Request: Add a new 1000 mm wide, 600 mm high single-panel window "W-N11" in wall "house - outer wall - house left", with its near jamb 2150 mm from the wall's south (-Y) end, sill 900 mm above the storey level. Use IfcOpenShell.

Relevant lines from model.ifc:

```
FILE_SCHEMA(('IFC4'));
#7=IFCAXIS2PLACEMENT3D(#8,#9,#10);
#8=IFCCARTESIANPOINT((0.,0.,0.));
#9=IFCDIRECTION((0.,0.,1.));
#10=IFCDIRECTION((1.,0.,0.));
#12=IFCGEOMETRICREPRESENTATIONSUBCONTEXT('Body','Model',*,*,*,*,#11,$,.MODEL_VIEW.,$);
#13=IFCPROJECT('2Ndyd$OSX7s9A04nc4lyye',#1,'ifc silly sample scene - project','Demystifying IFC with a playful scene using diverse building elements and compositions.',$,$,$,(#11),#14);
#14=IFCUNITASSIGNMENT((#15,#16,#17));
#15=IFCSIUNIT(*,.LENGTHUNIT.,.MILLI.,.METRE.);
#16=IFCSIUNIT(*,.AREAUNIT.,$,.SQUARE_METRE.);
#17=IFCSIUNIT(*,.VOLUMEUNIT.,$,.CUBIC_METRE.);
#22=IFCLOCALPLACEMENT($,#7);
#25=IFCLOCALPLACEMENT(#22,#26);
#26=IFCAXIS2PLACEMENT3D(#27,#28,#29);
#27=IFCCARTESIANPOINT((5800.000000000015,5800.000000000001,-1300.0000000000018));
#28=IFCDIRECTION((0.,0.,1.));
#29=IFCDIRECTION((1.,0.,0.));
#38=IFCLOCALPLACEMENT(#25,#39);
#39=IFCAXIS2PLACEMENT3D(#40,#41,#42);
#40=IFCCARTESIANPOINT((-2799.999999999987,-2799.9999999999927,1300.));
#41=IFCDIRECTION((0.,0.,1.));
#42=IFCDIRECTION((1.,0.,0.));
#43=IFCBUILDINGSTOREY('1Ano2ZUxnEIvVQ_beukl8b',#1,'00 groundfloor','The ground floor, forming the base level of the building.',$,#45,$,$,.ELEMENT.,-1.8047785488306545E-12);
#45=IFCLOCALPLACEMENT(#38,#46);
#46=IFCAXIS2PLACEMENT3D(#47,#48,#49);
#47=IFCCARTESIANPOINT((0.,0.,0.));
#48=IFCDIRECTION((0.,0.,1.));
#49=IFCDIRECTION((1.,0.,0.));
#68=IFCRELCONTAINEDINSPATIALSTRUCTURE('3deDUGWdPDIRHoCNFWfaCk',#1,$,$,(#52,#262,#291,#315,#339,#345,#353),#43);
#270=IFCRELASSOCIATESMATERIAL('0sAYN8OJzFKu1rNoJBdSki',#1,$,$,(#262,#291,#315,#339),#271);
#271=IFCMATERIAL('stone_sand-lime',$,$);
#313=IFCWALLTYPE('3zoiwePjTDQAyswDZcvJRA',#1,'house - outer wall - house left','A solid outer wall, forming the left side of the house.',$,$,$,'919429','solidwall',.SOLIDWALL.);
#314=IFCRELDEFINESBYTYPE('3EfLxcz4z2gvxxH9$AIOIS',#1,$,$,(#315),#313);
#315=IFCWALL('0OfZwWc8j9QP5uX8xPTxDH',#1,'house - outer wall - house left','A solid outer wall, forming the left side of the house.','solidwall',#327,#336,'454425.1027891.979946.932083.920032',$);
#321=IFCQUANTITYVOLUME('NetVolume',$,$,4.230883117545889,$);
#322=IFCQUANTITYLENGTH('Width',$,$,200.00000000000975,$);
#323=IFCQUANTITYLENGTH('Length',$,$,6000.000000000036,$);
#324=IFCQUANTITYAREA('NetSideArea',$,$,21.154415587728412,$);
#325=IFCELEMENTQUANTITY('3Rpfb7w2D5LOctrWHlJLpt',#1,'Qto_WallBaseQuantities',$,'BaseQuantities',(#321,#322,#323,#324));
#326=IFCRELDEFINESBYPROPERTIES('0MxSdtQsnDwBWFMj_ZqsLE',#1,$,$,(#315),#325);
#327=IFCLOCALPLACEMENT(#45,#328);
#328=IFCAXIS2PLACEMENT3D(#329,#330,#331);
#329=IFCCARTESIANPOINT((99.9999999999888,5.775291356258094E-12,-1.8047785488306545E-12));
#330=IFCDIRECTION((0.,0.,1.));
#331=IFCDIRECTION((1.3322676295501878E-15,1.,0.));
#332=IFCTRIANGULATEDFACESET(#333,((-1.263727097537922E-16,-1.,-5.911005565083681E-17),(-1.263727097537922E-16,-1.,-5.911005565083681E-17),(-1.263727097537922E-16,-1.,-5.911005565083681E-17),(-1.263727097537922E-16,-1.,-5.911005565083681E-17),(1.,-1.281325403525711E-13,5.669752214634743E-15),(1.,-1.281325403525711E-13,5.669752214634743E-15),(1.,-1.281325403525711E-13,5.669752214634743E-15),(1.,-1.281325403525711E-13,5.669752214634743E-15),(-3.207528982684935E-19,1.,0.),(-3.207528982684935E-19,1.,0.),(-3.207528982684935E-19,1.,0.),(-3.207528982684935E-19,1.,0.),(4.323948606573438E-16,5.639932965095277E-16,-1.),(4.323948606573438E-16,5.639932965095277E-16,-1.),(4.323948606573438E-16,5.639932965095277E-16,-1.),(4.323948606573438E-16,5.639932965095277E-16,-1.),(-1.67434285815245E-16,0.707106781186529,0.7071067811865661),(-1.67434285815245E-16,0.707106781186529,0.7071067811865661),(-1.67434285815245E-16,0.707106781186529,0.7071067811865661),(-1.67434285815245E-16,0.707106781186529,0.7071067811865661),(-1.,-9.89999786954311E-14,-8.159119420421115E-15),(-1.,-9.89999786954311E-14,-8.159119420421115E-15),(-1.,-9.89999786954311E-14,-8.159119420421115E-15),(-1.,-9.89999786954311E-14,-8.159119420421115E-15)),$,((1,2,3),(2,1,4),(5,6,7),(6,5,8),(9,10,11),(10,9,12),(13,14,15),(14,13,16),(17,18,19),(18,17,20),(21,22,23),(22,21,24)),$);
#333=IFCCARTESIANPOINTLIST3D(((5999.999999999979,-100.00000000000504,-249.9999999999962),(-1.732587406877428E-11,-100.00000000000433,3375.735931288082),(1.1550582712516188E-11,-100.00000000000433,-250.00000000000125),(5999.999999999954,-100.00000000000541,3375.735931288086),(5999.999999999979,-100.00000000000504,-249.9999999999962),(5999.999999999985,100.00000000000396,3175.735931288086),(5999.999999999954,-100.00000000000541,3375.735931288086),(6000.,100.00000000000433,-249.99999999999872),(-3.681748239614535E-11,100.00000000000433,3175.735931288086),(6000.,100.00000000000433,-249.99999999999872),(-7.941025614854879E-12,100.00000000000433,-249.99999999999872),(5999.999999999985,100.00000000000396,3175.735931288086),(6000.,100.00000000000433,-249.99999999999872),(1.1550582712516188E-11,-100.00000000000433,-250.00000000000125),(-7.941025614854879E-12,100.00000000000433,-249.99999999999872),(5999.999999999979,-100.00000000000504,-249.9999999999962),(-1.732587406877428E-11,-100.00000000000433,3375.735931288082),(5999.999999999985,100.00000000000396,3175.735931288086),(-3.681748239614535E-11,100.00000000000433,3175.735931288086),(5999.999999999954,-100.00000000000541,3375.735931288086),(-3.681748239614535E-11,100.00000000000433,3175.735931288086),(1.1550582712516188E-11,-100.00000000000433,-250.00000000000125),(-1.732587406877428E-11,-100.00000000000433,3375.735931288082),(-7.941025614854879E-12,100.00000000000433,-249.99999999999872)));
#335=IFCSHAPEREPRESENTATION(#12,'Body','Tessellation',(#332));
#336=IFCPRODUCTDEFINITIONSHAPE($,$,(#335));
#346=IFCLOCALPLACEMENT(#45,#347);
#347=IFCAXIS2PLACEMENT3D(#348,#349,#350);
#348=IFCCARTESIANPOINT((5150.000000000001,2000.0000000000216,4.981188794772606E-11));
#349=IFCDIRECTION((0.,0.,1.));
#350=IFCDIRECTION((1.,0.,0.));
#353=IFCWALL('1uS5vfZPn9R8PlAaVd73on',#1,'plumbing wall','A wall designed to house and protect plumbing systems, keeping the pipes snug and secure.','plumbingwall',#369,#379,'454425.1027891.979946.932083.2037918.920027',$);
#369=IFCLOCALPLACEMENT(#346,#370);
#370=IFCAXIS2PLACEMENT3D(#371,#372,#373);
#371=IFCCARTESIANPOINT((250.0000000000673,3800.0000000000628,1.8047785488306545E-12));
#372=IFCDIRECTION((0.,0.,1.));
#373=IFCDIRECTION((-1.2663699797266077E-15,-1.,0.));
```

```python
import numpy as np
import ifcopenshell
import ifcopenshell.api.feature
import ifcopenshell.api.geometry
import ifcopenshell.api.pset
import ifcopenshell.api.root
import ifcopenshell.api.spatial
import ifcopenshell.geom
import ifcopenshell.util.element
import ifcopenshell.util.placement
import ifcopenshell.util.representation
import ifcopenshell.util.shape
import ifcopenshell.util.unit

model = ifcopenshell.open("model.ifc")
unit_scale = ifcopenshell.util.unit.calculate_unit_scale(model)
area_scale = ifcopenshell.util.unit.calculate_unit_scale(model, "AREAUNIT")
volume_scale = ifcopenshell.util.unit.calculate_unit_scale(model, "VOLUMEUNIT")
settings = ifcopenshell.geom.settings()


def volume(element):
    """Net volume in cubic metres, openings subtracted."""
    shape = ifcopenshell.geom.create_shape(settings, element)
    return ifcopenshell.util.shape.get_volume(shape.geometry)


wall = model.by_guid("0OfZwWc8j9QP5uX8xPTxDH")
storey = ifcopenshell.util.element.get_container(wall, ifc_class="IfcBuildingStorey")
context = ifcopenshell.util.representation.get_context(model, "Model", "Body", "MODEL_VIEW")
before = volume(wall)

width, height, from_end, sill = 1, 0.6, 2.15, 0.9  # metres

# The wall runs along its own X axis, and the end named is its -X end.
wall_shape = ifcopenshell.geom.create_shape(settings, wall)
x, y, z = ifcopenshell.util.shape.get_vertices(wall_shape.geometry).T
start = x.min() + from_end
face, thickness = float(y.min()), float(y.max() - y.min())
wall_matrix = ifcopenshell.util.placement.get_local_placement(wall.ObjectPlacement)
level = ifcopenshell.util.placement.get_local_placement(storey.ObjectPlacement)[2, 3]


def in_wall(x, y):
    """Placement at x, y metres in the wall's axes, at sill height."""
    matrix = wall_matrix.copy()
    matrix[:, 3] = wall_matrix @ np.array([x / unit_scale, y / unit_scale, 0.0, 1.0])
    matrix[2, 3] = level + sill / unit_scale
    return matrix


# Opening: a box that overshoots both wall faces by 50 mm.
opening = ifcopenshell.api.root.create_entity(model, ifc_class="IfcOpeningElement", predefined_type="OPENING")
box = ifcopenshell.api.geometry.add_wall_representation(
    model, context=context, length=width, height=height, thickness=thickness + 0.1
)
ifcopenshell.api.geometry.assign_representation(model, product=opening, representation=box)
ifcopenshell.api.geometry.edit_object_placement(model, product=opening, matrix=in_wall(start, face - 0.05), is_si=False)
ifcopenshell.api.feature.add_feature(model, feature=opening, element=wall)

window = ifcopenshell.api.root.create_entity(model, ifc_class="IfcWindow", name="W-N11", predefined_type="WINDOW")
window.OverallWidth, window.OverallHeight = width / unit_scale, height / unit_scale
window.PartitioningType = "SINGLE_PANEL"
body = ifcopenshell.api.geometry.add_window_representation(
    model,
    context=context,
    overall_width=window.OverallWidth,
    overall_height=window.OverallHeight,
    partition_type="SINGLE_PANEL",
)
ifcopenshell.api.geometry.assign_representation(model, product=window, representation=body)
ifcopenshell.api.spatial.assign_container(model, products=[window], relating_structure=storey)
ifcopenshell.api.feature.add_filling(model, opening=opening, element=window)

# Centre the window in the wall's thickness.
ifcopenshell.api.geometry.edit_object_placement(model, product=window, matrix=in_wall(start, face), is_si=False)
window_shape = ifcopenshell.geom.create_shape(settings, window)
depth = ifcopenshell.util.shape.get_vertices(window_shape.geometry)[:, 1]
offset = face + thickness / 2 - (depth.min() + depth.max()) / 2
ifcopenshell.api.geometry.edit_object_placement(model, product=window, matrix=in_wall(start, offset), is_si=False)

after = volume(wall)

# Update the wall's stored quantities.
qto = model.by_id(ifcopenshell.util.element.get_pset(wall, "Qto_WallBaseQuantities", should_inherit=False)["id"])
ifcopenshell.api.pset.edit_qto(model, qto=qto, properties={
    "NetVolume": after / volume_scale,
    "NetSideArea": after / thickness / area_scale,
})

print(f"wall volume {before:.3f} -> {after:.3f} m3")

model.write("model_updated.ifc")
```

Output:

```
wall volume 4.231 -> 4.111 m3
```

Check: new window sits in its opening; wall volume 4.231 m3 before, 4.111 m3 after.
